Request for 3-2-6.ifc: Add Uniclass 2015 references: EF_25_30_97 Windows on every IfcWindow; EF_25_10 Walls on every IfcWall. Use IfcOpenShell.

First a look at what the model holds.

```python
import ifcopenshell

model = ifcopenshell.open("3-2-6.ifc")
print(model.schema)
print("classifications:", [c.Name for c in model.by_type("IfcClassification")])
for ifc_class in ("IfcDoor", "IfcRoof", "IfcStair", "IfcWall", "IfcWindow"):
    print(ifc_class, len(model.by_type(ifc_class)))
```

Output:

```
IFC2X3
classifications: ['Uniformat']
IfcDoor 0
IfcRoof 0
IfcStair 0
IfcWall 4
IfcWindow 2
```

```python
import ifcopenshell
import ifcopenshell.api.classification

model = ifcopenshell.open("3-2-6.ifc")

# IFC2X3 requires Source and Edition and has no link from the project to the system.
system = model.create_entity("IfcClassification", Source="NBS", Edition="2015", Name="Uniclass 2015")

codes = {
    "IfcWindow": ("EF_25_30_97", "Windows"),
    "IfcWall": ("EF_25_10", "Walls"),
}
for ifc_class, (code, name) in codes.items():
    products = model.by_type(ifc_class)
    ifcopenshell.api.classification.add_reference(
        model, products=products, classification=system, identification=code, name=name
    )
    print(code, len(products))

model.write("3-2-6_rev.ifc")
```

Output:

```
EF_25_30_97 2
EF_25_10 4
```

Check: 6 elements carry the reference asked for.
